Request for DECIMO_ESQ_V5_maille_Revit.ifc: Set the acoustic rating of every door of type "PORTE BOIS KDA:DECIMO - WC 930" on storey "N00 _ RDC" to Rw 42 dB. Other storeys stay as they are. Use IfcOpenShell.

First a look at what the model holds.

```python
import ifcopenshell
import ifcopenshell.util.element

model = ifcopenshell.open("DECIMO_ESQ_V5_maille_Revit.ifc")
print(model.schema)
storey = next(s for s in model.by_type("IfcBuildingStorey") if s.Name == "N00 _ RDC")
doors = [e for e in ifcopenshell.util.element.get_decomposition(storey) if e.is_a("IfcDoor")]
seen = {}
for e in doors:
    element_type = ifcopenshell.util.element.get_type(e)
    key = (element_type.Name if element_type != e and element_type else None, ifcopenshell.util.element.get_pset(e, "Pset_DoorCommon", "AcousticRating"))
    seen[key] = seen.get(key, 0) + 1
for (name, value), count in sorted(seen.items(), key=str):
    print(count, "x", name, "|", value)
```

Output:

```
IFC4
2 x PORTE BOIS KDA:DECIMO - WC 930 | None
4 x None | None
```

```python
import ifcopenshell
import ifcopenshell.api.pset
import ifcopenshell.util.element

model = ifcopenshell.open("DECIMO_ESQ_V5_maille_Revit.ifc")

storey = next(s for s in model.by_type("IfcBuildingStorey") if s.Name == "N00 _ RDC")
doors = [e for e in ifcopenshell.util.element.get_decomposition(storey) if e.is_a("IfcDoor")]

count = 0
for e in doors:
    element_type = ifcopenshell.util.element.get_type(e)
    if element_type in (None, e) or element_type.Name != "PORTE BOIS KDA:DECIMO - WC 930":
        continue
    # add_pset returns the element's existing set when there is one.
    pset = ifcopenshell.api.pset.add_pset(model, product=e, name="Pset_DoorCommon")
    ifcopenshell.api.pset.edit_pset(model, pset=pset, properties={"AcousticRating": "Rw 42 dB"})
    count += 1

print(count, "doors updated")

model.write("DECIMO_ESQ_V5_maille_Revit_edited.ifc")
```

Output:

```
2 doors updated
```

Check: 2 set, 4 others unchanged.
